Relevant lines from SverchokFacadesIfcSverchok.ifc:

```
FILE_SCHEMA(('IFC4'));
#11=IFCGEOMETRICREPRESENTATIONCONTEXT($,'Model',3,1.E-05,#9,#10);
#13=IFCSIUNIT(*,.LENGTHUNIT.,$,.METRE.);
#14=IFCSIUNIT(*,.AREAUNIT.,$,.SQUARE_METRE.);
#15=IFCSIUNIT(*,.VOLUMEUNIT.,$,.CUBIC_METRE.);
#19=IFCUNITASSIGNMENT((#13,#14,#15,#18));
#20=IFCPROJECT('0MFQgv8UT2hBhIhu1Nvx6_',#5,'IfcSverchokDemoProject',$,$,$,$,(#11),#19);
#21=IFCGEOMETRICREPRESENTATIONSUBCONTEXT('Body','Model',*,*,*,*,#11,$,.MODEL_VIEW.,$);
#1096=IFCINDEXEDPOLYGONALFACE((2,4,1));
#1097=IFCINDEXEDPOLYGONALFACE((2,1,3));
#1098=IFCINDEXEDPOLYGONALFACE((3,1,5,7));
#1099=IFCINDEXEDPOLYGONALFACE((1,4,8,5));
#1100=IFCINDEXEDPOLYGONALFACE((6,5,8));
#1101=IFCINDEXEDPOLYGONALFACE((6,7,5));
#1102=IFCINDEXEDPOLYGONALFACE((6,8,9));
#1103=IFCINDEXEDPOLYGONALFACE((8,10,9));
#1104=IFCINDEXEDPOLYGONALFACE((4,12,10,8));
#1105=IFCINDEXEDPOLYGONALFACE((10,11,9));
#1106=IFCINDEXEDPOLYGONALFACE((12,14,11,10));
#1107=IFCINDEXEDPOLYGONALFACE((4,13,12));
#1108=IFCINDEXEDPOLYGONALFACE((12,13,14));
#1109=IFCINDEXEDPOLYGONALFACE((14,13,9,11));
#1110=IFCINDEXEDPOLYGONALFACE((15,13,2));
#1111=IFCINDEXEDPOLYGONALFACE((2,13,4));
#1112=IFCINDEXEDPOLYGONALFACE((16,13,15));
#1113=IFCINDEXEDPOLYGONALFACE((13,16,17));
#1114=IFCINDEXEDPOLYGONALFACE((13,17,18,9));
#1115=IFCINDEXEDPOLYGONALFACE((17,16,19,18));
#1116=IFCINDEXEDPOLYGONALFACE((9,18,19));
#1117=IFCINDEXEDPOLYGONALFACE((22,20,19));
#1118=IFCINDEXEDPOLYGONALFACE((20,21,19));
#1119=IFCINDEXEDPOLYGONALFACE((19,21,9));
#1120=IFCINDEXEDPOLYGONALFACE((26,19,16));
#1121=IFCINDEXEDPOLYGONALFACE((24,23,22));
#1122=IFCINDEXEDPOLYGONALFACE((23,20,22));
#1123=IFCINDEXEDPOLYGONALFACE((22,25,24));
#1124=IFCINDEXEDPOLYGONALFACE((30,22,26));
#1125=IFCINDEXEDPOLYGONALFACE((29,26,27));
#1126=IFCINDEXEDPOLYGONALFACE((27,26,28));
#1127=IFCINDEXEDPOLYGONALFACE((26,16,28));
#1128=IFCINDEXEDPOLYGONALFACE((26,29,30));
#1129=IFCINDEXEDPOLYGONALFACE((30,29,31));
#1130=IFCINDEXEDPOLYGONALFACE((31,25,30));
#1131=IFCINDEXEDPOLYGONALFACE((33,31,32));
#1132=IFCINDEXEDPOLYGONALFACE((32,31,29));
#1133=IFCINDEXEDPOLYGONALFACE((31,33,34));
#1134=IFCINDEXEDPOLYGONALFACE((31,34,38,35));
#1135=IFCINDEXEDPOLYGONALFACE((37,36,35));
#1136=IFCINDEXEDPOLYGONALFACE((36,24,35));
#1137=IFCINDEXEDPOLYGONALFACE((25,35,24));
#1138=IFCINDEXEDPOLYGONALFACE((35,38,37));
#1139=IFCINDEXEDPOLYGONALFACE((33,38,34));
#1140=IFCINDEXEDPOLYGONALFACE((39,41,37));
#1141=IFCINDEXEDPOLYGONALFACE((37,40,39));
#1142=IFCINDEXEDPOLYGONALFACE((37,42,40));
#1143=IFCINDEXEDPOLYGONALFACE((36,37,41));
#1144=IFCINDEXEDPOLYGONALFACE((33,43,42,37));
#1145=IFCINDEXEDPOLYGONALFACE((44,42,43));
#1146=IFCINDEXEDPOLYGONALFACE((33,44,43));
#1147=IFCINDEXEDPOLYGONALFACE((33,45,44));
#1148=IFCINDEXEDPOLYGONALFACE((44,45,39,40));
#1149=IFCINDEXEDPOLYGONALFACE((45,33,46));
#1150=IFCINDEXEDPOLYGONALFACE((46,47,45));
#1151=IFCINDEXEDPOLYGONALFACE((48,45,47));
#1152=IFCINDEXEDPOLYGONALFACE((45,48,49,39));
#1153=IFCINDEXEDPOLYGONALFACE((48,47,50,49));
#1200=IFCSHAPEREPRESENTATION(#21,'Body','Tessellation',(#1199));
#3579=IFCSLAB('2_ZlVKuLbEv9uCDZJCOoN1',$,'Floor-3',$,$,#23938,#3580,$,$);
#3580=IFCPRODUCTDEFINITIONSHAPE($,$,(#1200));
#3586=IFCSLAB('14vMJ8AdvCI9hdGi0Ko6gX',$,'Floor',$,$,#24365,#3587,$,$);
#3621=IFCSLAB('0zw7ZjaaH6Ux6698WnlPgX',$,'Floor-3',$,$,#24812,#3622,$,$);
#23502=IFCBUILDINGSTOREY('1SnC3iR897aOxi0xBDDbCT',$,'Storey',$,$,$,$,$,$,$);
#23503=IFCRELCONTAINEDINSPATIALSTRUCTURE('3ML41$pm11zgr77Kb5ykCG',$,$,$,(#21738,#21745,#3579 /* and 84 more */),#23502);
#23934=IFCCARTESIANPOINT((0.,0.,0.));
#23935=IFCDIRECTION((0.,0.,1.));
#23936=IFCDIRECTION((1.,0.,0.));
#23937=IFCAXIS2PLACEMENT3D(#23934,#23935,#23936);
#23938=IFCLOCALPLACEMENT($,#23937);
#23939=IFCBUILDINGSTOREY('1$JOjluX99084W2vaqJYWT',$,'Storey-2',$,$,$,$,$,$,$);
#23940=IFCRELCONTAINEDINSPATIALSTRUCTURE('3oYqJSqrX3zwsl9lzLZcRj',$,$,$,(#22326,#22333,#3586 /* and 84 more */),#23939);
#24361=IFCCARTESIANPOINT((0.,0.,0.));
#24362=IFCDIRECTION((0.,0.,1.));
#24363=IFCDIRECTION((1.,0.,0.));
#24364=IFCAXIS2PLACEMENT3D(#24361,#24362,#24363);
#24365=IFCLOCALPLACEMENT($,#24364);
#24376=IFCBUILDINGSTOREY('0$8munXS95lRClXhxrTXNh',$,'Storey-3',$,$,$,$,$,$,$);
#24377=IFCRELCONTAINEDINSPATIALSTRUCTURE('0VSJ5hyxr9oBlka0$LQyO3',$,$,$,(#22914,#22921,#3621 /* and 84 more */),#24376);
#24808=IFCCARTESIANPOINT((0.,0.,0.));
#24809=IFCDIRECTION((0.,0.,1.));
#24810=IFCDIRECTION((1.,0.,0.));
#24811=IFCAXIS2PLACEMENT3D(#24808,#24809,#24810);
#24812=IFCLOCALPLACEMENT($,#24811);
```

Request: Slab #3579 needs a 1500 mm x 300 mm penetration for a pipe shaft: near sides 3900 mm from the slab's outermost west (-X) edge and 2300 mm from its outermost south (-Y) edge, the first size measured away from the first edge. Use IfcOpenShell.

```python
import numpy as np
import ifcopenshell
import ifcopenshell.api.feature
import ifcopenshell.api.geometry
import ifcopenshell.api.root
import ifcopenshell.geom
import ifcopenshell.util.placement
import ifcopenshell.util.representation
import ifcopenshell.util.shape
import ifcopenshell.util.unit

model = ifcopenshell.open("SverchokFacadesIfcSverchok.ifc")
unit_scale = ifcopenshell.util.unit.calculate_unit_scale(model)
settings = ifcopenshell.geom.settings()


def volume(element):
    """Net volume in cubic metres, openings subtracted."""
    shape = ifcopenshell.geom.create_shape(settings, element)
    return ifcopenshell.util.shape.get_volume(shape.geometry)


slab = model.by_guid("2_ZlVKuLbEv9uCDZJCOoN1")
before = volume(slab)

# Extent in the slab's own axes, in metres. The edges named are its -X and -Y sides.
slab_shape = ifcopenshell.geom.create_shape(settings, slab)
vertices = ifcopenshell.util.shape.get_vertices(slab_shape.geometry)
x_min, y_min, bottom = vertices.min(axis=0)
top = vertices[:, 2].max()

opening = ifcopenshell.api.root.create_entity(model, ifc_class="IfcOpeningElement", name="Pipe shaft opening", predefined_type="OPENING")
context = ifcopenshell.util.representation.get_context(model, "Model", "Body", "MODEL_VIEW")
width, depth = 1.5, 0.3
outline = [(0.0, 0.0), (width, 0.0), (width, depth), (0.0, depth), (0.0, 0.0)]
# Overshoot both faces by 50 mm so the cut is clean.
shape = ifcopenshell.api.geometry.add_slab_representation(
    model, context=context, depth=top - bottom + 0.1, polyline=outline
)
ifcopenshell.api.geometry.assign_representation(model, product=opening, representation=shape)

matrix = ifcopenshell.util.placement.get_local_placement(slab.ObjectPlacement)
matrix[:, 3] = matrix @ np.append(np.array([x_min + 3.9, y_min + 2.3, bottom - 0.05]) / unit_scale, 1.0)
ifcopenshell.api.geometry.edit_object_placement(model, product=opening, matrix=matrix, is_si=False)
ifcopenshell.api.feature.add_feature(model, feature=opening, element=slab)

after = volume(slab)

print(f"slab volume {before:.3f} -> {after:.3f} m3")

model.write("SverchokFacadesIfcSverchok_updated.ifc")
```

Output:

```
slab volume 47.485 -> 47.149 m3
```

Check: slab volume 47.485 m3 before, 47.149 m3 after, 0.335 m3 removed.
